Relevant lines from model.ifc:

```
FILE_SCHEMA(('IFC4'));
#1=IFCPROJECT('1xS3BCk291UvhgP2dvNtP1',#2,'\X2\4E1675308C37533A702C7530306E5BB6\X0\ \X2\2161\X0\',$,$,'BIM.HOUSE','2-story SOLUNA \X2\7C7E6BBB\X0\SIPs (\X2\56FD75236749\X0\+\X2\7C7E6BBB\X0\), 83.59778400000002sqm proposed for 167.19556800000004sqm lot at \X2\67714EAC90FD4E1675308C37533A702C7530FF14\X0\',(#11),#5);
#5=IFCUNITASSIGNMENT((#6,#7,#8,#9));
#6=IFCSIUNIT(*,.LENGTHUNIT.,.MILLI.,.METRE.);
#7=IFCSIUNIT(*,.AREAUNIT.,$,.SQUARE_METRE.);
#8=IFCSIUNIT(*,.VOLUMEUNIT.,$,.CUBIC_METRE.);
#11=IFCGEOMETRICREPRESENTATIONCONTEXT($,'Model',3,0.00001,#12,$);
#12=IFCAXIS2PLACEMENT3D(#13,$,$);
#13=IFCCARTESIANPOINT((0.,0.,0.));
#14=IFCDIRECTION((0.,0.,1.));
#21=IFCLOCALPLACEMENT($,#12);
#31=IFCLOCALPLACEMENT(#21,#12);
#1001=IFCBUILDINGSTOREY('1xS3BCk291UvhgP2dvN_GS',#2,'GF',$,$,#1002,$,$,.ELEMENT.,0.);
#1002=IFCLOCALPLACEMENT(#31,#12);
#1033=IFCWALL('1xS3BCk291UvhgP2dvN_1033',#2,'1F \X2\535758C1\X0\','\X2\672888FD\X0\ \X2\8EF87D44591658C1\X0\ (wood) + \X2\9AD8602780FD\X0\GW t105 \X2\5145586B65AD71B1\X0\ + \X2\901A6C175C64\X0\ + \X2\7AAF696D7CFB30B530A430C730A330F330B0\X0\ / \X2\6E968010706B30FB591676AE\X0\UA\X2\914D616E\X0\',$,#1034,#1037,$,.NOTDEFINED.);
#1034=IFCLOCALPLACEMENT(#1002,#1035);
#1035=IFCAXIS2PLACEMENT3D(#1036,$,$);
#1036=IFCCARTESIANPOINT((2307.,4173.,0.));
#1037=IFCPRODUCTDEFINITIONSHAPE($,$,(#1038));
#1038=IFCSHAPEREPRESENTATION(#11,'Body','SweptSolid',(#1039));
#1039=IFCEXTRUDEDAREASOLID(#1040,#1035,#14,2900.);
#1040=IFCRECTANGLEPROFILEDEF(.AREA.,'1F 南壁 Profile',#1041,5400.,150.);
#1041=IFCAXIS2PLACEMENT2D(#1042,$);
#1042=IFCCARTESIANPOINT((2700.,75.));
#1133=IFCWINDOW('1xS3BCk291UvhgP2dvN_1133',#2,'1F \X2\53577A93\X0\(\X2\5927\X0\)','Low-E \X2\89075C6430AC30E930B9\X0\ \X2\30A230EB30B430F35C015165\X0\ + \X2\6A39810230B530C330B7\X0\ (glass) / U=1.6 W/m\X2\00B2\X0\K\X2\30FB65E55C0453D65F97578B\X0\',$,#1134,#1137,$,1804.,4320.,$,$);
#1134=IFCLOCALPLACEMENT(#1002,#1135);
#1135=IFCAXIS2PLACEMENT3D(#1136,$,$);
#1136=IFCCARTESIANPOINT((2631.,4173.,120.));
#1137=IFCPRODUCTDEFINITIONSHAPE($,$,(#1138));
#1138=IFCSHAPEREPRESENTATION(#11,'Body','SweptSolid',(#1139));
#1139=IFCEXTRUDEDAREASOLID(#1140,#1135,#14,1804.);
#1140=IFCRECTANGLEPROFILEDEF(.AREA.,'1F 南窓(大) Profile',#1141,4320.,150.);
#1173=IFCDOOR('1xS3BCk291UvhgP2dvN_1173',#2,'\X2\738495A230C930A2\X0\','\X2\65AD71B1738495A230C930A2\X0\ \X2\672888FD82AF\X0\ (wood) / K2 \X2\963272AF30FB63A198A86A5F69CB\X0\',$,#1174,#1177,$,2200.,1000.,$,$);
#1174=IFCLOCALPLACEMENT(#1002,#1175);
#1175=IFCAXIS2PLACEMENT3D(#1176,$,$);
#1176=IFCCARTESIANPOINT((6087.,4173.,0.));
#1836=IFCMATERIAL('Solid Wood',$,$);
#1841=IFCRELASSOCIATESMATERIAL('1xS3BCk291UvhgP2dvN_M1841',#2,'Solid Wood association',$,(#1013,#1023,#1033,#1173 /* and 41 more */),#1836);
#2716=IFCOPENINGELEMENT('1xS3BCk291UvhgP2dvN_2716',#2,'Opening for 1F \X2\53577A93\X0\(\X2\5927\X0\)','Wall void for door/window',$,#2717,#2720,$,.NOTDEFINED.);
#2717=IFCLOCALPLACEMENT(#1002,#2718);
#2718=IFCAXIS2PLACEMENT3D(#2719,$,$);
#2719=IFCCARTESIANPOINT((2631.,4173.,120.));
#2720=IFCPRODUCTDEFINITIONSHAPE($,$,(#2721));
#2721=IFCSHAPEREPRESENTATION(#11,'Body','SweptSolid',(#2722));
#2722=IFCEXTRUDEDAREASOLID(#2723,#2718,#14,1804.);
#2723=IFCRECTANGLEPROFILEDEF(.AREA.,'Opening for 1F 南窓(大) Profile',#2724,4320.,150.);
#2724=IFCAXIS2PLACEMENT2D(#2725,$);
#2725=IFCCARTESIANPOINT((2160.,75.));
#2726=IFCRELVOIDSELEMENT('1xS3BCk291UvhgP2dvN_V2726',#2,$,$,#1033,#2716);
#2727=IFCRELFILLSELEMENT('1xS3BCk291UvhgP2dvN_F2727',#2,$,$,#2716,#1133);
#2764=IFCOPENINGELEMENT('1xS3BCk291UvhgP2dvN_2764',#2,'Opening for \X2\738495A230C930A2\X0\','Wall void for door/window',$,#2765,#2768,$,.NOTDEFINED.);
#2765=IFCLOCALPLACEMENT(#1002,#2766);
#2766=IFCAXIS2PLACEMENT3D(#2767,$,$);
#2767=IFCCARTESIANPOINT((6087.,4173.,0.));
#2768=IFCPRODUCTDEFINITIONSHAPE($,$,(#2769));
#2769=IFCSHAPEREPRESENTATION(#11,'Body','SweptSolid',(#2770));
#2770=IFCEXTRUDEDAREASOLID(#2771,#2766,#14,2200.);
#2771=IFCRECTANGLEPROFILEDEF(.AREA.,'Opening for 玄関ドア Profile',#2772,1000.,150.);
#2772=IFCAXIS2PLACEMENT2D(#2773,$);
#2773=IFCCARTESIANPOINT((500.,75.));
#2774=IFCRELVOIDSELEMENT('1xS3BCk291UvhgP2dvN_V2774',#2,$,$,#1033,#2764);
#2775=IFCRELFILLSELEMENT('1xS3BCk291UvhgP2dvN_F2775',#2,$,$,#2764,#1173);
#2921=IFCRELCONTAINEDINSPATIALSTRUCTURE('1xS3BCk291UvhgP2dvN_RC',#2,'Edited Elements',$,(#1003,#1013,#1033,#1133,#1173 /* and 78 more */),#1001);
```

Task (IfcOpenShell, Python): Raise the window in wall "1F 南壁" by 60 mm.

```python
import numpy as np
import ifcopenshell
import ifcopenshell.api.geometry
import ifcopenshell.util.placement
import ifcopenshell.util.unit

model = ifcopenshell.open("model.ifc")
unit_scale = ifcopenshell.util.unit.calculate_unit_scale(model)

window = model.by_id(1133)
opening = window.FillsVoids[0].RelatingOpeningElement
dz = 60.0

shift = np.array([0.0, 0.0, dz])
# The window is not placed relative to its opening, so move both.
for product in (opening, window):
    matrix = ifcopenshell.util.placement.get_local_placement(product.ObjectPlacement)
    matrix[:3, 3] += shift
    ifcopenshell.api.geometry.edit_object_placement(model, product=product, matrix=matrix, is_si=False)

print(f"moved by {dz * unit_scale:+.3f} m")

model.write("model-out.ifc")
```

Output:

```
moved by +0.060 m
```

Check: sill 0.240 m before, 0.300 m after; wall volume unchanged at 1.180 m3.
